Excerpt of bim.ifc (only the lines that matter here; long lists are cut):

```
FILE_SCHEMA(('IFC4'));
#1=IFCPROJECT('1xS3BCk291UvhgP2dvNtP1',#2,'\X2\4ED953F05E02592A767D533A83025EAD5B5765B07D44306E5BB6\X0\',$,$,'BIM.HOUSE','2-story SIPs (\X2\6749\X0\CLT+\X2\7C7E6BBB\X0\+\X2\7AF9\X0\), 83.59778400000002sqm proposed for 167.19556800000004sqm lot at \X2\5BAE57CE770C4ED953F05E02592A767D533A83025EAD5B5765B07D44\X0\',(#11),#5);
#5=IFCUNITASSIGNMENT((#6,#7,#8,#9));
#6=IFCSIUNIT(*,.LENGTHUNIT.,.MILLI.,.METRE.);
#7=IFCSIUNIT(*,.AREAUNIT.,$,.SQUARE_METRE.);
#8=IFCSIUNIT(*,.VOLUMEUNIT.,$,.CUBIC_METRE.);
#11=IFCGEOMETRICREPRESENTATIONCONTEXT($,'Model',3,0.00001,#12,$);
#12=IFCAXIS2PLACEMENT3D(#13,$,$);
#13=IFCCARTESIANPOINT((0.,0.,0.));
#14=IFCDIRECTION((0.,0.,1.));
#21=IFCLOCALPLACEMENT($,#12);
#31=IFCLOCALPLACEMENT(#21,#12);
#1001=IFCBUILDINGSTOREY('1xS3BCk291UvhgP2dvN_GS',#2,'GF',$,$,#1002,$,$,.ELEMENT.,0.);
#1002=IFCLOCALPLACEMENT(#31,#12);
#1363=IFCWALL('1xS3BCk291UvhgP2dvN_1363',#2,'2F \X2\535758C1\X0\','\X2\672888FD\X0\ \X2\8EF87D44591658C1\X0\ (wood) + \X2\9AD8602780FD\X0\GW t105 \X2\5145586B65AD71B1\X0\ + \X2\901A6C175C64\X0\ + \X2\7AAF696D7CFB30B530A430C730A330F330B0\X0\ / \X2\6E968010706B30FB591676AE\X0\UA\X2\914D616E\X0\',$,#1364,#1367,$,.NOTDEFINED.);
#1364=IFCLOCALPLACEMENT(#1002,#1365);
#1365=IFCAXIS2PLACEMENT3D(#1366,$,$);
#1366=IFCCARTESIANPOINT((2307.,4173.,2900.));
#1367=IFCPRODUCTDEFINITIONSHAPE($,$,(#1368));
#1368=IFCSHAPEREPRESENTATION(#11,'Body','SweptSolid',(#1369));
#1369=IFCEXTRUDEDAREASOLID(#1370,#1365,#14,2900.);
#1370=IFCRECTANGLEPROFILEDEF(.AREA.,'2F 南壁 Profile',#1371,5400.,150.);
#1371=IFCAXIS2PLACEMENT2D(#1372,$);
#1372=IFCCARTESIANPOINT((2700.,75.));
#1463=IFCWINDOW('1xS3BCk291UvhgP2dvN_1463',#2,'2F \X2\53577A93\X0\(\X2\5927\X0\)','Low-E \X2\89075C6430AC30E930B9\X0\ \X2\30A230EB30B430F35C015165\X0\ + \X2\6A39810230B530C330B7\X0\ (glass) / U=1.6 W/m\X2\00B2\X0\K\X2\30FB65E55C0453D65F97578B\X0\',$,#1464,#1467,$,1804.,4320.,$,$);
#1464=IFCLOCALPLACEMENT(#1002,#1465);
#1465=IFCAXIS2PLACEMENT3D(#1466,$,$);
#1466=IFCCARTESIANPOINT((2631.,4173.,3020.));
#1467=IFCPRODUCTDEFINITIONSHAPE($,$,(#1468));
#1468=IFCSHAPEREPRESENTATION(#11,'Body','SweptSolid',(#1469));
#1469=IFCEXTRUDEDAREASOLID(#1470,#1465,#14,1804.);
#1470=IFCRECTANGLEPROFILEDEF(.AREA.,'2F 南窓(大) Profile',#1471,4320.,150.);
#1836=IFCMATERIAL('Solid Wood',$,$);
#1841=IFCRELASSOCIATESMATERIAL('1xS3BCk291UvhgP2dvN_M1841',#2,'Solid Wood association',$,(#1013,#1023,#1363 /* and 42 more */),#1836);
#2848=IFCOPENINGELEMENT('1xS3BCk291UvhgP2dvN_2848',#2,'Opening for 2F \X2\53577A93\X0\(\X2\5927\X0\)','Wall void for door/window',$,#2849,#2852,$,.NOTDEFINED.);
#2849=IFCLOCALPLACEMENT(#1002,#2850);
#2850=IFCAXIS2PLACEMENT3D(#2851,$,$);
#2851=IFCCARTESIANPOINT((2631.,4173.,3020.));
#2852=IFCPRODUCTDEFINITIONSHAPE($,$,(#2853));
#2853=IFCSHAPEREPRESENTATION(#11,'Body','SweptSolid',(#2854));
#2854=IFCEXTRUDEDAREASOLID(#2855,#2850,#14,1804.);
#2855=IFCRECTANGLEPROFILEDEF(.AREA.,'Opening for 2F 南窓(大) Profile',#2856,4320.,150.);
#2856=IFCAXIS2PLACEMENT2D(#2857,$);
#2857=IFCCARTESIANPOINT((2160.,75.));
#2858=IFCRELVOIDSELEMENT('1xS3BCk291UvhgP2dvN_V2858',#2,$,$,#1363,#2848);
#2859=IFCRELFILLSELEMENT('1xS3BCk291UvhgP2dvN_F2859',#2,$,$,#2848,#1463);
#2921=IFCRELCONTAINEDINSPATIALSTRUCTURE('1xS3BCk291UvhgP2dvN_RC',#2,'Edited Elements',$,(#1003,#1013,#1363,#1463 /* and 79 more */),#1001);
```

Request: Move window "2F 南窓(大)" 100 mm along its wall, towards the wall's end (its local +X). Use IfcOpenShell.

```python
import ifcopenshell
import ifcopenshell.api.geometry
import ifcopenshell.util.placement

model = ifcopenshell.open("bim.ifc")

window = model.by_id(1463)
opening = window.FillsVoids[0].RelatingOpeningElement
wall = opening.VoidsElements[0].RelatingBuildingElement

wall_matrix = ifcopenshell.util.placement.get_local_placement(wall.ObjectPlacement)
shift = wall_matrix[:3, 0] * 100.0
before = ifcopenshell.util.placement.get_local_placement(window.ObjectPlacement)[:3, 3].copy()

# The window is not placed relative to its opening, so move both.
for product in (opening, window):
    matrix = ifcopenshell.util.placement.get_local_placement(product.ObjectPlacement)
    matrix[:3, 3] += shift
    ifcopenshell.api.geometry.edit_object_placement(model, product=product, matrix=matrix, is_si=False)

after = ifcopenshell.util.placement.get_local_placement(window.ObjectPlacement)[:3, 3]
print("window moved by", (after - before).round(3) + 0.0)

model.write("bim_edited.ifc")
```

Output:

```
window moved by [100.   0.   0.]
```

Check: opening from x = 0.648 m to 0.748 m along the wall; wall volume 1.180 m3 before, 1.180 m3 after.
